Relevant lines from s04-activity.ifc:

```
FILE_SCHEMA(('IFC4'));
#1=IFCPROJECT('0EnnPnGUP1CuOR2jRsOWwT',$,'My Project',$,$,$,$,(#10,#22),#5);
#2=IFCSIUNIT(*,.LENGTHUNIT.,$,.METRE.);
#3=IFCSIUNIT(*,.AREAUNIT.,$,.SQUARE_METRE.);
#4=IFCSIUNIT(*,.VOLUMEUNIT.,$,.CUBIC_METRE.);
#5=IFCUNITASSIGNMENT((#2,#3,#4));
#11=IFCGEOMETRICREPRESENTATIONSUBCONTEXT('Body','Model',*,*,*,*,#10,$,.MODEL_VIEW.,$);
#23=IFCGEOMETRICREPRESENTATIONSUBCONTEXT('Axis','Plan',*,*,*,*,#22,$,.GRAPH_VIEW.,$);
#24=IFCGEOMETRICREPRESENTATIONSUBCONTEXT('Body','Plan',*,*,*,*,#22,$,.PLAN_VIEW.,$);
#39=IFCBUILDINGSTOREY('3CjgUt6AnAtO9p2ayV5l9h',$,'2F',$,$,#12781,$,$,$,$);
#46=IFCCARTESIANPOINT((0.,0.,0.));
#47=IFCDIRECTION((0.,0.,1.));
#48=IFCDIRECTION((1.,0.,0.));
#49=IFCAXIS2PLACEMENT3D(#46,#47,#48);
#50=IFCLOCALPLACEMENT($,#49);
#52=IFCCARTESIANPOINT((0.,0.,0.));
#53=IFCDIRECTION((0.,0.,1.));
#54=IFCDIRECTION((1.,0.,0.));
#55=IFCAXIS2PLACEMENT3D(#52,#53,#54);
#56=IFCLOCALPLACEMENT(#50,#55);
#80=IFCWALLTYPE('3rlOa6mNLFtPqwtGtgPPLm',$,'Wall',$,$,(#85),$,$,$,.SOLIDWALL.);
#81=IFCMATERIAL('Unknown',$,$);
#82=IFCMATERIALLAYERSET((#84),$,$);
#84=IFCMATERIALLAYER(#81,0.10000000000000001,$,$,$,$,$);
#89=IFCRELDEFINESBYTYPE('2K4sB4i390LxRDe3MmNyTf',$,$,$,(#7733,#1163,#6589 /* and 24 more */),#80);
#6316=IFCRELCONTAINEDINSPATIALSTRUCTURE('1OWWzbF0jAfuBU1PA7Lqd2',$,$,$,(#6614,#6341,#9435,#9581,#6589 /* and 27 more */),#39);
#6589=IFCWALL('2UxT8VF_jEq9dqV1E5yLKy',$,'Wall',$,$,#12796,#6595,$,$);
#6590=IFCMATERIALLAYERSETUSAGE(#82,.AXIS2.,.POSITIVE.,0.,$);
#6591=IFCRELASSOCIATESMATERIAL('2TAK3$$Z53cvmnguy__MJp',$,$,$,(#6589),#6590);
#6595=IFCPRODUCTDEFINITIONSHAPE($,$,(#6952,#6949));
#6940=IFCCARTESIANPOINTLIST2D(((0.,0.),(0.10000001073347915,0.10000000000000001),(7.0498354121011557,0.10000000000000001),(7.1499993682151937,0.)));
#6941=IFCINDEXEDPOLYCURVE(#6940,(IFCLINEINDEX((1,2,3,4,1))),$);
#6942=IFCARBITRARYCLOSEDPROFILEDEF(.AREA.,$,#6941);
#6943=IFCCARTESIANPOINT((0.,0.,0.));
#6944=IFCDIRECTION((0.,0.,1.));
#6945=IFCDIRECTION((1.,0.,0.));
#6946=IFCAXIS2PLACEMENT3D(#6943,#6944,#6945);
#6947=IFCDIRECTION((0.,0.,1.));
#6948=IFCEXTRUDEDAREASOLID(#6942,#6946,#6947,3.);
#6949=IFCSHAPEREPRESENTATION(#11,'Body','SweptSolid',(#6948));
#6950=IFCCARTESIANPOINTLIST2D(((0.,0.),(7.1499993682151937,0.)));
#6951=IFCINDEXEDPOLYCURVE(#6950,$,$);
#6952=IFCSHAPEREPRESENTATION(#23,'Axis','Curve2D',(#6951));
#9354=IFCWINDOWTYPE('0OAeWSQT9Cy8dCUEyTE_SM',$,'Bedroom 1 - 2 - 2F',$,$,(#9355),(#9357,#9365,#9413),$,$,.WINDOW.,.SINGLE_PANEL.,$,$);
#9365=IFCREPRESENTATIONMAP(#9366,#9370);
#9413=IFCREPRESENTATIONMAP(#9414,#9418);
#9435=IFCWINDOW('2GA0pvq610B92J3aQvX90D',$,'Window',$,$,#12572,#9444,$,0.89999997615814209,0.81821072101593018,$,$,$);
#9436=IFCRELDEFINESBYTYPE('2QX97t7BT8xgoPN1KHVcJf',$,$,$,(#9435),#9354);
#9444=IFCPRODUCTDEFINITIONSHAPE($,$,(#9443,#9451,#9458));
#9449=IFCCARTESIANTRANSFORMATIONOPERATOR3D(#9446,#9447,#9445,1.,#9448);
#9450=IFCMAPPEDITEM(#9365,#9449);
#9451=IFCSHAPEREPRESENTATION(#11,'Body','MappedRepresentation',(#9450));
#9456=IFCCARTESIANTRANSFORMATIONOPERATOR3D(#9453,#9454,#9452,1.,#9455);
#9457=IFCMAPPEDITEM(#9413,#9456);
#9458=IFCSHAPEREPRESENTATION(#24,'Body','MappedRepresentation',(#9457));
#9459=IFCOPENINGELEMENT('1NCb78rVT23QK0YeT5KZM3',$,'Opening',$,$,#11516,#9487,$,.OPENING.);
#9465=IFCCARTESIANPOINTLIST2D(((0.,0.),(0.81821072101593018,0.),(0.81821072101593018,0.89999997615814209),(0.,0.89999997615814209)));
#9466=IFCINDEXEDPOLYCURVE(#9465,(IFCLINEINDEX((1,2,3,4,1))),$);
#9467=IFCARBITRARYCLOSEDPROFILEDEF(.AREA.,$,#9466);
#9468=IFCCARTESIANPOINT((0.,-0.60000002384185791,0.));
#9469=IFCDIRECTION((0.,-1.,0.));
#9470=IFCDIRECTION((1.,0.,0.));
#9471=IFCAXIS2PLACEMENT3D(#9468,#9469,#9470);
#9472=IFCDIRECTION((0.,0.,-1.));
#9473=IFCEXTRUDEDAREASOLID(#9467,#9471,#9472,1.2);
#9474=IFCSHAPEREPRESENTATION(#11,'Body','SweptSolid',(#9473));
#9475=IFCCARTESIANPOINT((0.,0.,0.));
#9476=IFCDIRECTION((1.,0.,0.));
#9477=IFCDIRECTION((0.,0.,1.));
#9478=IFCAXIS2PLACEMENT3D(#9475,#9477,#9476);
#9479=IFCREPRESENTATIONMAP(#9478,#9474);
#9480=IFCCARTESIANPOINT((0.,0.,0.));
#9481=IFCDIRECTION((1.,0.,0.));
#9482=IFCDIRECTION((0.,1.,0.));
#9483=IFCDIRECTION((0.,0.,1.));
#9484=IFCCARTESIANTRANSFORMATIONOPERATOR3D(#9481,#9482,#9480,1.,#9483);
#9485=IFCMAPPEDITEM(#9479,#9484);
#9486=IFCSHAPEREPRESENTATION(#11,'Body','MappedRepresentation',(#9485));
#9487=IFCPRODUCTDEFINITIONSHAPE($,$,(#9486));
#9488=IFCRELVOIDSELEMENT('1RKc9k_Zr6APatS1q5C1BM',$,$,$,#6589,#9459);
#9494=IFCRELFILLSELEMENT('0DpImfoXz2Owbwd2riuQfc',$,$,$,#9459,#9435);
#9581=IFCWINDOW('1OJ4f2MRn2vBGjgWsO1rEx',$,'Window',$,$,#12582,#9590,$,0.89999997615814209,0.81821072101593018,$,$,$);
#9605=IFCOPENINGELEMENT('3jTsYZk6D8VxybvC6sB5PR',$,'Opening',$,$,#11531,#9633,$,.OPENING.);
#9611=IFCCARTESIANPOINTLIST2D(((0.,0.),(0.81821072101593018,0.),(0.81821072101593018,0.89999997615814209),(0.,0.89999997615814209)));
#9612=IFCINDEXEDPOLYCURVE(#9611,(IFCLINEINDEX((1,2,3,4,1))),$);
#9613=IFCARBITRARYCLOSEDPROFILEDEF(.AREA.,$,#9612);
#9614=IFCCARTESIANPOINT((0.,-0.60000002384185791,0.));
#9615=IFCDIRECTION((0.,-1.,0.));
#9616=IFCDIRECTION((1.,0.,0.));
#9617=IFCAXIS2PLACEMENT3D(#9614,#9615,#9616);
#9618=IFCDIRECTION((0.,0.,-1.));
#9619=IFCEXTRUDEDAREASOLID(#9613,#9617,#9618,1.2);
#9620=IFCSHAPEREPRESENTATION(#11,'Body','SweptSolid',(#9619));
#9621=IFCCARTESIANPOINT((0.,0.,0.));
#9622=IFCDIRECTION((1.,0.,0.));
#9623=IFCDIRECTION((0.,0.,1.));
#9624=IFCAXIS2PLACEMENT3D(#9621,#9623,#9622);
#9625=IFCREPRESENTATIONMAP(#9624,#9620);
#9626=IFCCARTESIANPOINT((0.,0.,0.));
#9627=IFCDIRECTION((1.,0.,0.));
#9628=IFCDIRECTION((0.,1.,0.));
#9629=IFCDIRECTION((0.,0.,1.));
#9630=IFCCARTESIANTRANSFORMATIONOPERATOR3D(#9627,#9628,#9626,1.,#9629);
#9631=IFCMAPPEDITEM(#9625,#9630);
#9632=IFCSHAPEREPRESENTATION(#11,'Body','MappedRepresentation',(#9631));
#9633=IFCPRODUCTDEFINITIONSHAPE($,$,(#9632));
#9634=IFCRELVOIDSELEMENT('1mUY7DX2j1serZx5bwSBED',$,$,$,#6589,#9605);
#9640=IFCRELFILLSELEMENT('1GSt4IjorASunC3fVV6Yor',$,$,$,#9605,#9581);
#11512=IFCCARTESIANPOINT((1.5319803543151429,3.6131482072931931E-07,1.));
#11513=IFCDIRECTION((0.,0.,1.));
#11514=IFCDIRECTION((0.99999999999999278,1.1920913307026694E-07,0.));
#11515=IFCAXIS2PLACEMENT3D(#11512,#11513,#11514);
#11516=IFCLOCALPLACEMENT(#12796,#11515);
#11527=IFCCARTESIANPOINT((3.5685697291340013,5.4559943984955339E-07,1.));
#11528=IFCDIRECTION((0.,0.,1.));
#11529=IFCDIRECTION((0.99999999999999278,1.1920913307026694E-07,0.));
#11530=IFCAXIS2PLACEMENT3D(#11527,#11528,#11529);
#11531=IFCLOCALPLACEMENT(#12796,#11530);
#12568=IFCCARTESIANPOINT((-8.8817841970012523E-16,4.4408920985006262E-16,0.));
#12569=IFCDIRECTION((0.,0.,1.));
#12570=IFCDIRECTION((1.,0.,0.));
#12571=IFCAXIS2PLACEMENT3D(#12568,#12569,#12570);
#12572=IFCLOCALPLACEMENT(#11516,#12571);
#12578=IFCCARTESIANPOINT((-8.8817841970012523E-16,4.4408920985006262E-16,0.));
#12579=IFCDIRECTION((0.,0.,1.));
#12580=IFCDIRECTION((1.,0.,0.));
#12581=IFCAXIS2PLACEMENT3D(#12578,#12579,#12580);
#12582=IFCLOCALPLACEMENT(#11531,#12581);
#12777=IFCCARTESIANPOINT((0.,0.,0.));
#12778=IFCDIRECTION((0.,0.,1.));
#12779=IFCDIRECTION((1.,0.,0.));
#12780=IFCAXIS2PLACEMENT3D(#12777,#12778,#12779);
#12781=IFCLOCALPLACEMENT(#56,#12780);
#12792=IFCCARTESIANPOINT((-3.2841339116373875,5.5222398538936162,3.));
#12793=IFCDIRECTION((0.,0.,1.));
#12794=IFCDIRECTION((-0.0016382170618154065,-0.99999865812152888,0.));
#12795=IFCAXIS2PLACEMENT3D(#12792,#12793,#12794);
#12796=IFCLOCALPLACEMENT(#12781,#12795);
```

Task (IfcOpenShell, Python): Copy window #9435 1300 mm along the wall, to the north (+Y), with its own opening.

```python
import ifcopenshell
import ifcopenshell.api.feature
import ifcopenshell.api.geometry
import ifcopenshell.api.root
import ifcopenshell.geom
import ifcopenshell.util.element
import ifcopenshell.util.placement
import ifcopenshell.util.shape
import ifcopenshell.util.unit

model = ifcopenshell.open("s04-activity.ifc")
unit_scale = ifcopenshell.util.unit.calculate_unit_scale(model)
settings = ifcopenshell.geom.settings()


def volume(element):
    """Net volume in cubic metres, openings subtracted."""
    shape = ifcopenshell.geom.create_shape(settings, element)
    return ifcopenshell.util.shape.get_volume(shape.geometry)


window = model.by_guid("2GA0pvq610B92J3aQvX90D")
opening = window.FillsVoids[0].RelatingOpeningElement
wall = opening.VoidsElements[0].RelatingBuildingElement
before = volume(wall)
shift = ifcopenshell.util.placement.get_local_placement(wall.ObjectPlacement)[:3, 0] * -1.3 / unit_scale

# copy_class copies the void relationship, type, container and properties, but no geometry.
new_opening = ifcopenshell.api.root.copy_class(model, product=opening)
new_opening.Representation = ifcopenshell.util.element.copy_deep(
    model, opening.Representation, exclude=["IfcGeometricRepresentationContext", "IfcRepresentationMap"]
)
new_window = ifcopenshell.api.root.copy_class(model, product=window)
new_window.Representation = ifcopenshell.util.element.copy_deep(
    model, window.Representation, exclude=["IfcGeometricRepresentationContext", "IfcRepresentationMap"]
)
ifcopenshell.api.feature.add_filling(model, opening=new_opening, element=new_window)

for old, new in ((opening, new_opening), (window, new_window)):
    matrix = ifcopenshell.util.placement.get_local_placement(old.ObjectPlacement)
    matrix[:3, 3] += shift
    ifcopenshell.api.geometry.edit_object_placement(model, product=new, matrix=matrix, is_si=False)

after = volume(wall)

print(f"wall volume {before:.3f} -> {after:.3f} m3")

model.write("s04-activity_rev.ifc")
```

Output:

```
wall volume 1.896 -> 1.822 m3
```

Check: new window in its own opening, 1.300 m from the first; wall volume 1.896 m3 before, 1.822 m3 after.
